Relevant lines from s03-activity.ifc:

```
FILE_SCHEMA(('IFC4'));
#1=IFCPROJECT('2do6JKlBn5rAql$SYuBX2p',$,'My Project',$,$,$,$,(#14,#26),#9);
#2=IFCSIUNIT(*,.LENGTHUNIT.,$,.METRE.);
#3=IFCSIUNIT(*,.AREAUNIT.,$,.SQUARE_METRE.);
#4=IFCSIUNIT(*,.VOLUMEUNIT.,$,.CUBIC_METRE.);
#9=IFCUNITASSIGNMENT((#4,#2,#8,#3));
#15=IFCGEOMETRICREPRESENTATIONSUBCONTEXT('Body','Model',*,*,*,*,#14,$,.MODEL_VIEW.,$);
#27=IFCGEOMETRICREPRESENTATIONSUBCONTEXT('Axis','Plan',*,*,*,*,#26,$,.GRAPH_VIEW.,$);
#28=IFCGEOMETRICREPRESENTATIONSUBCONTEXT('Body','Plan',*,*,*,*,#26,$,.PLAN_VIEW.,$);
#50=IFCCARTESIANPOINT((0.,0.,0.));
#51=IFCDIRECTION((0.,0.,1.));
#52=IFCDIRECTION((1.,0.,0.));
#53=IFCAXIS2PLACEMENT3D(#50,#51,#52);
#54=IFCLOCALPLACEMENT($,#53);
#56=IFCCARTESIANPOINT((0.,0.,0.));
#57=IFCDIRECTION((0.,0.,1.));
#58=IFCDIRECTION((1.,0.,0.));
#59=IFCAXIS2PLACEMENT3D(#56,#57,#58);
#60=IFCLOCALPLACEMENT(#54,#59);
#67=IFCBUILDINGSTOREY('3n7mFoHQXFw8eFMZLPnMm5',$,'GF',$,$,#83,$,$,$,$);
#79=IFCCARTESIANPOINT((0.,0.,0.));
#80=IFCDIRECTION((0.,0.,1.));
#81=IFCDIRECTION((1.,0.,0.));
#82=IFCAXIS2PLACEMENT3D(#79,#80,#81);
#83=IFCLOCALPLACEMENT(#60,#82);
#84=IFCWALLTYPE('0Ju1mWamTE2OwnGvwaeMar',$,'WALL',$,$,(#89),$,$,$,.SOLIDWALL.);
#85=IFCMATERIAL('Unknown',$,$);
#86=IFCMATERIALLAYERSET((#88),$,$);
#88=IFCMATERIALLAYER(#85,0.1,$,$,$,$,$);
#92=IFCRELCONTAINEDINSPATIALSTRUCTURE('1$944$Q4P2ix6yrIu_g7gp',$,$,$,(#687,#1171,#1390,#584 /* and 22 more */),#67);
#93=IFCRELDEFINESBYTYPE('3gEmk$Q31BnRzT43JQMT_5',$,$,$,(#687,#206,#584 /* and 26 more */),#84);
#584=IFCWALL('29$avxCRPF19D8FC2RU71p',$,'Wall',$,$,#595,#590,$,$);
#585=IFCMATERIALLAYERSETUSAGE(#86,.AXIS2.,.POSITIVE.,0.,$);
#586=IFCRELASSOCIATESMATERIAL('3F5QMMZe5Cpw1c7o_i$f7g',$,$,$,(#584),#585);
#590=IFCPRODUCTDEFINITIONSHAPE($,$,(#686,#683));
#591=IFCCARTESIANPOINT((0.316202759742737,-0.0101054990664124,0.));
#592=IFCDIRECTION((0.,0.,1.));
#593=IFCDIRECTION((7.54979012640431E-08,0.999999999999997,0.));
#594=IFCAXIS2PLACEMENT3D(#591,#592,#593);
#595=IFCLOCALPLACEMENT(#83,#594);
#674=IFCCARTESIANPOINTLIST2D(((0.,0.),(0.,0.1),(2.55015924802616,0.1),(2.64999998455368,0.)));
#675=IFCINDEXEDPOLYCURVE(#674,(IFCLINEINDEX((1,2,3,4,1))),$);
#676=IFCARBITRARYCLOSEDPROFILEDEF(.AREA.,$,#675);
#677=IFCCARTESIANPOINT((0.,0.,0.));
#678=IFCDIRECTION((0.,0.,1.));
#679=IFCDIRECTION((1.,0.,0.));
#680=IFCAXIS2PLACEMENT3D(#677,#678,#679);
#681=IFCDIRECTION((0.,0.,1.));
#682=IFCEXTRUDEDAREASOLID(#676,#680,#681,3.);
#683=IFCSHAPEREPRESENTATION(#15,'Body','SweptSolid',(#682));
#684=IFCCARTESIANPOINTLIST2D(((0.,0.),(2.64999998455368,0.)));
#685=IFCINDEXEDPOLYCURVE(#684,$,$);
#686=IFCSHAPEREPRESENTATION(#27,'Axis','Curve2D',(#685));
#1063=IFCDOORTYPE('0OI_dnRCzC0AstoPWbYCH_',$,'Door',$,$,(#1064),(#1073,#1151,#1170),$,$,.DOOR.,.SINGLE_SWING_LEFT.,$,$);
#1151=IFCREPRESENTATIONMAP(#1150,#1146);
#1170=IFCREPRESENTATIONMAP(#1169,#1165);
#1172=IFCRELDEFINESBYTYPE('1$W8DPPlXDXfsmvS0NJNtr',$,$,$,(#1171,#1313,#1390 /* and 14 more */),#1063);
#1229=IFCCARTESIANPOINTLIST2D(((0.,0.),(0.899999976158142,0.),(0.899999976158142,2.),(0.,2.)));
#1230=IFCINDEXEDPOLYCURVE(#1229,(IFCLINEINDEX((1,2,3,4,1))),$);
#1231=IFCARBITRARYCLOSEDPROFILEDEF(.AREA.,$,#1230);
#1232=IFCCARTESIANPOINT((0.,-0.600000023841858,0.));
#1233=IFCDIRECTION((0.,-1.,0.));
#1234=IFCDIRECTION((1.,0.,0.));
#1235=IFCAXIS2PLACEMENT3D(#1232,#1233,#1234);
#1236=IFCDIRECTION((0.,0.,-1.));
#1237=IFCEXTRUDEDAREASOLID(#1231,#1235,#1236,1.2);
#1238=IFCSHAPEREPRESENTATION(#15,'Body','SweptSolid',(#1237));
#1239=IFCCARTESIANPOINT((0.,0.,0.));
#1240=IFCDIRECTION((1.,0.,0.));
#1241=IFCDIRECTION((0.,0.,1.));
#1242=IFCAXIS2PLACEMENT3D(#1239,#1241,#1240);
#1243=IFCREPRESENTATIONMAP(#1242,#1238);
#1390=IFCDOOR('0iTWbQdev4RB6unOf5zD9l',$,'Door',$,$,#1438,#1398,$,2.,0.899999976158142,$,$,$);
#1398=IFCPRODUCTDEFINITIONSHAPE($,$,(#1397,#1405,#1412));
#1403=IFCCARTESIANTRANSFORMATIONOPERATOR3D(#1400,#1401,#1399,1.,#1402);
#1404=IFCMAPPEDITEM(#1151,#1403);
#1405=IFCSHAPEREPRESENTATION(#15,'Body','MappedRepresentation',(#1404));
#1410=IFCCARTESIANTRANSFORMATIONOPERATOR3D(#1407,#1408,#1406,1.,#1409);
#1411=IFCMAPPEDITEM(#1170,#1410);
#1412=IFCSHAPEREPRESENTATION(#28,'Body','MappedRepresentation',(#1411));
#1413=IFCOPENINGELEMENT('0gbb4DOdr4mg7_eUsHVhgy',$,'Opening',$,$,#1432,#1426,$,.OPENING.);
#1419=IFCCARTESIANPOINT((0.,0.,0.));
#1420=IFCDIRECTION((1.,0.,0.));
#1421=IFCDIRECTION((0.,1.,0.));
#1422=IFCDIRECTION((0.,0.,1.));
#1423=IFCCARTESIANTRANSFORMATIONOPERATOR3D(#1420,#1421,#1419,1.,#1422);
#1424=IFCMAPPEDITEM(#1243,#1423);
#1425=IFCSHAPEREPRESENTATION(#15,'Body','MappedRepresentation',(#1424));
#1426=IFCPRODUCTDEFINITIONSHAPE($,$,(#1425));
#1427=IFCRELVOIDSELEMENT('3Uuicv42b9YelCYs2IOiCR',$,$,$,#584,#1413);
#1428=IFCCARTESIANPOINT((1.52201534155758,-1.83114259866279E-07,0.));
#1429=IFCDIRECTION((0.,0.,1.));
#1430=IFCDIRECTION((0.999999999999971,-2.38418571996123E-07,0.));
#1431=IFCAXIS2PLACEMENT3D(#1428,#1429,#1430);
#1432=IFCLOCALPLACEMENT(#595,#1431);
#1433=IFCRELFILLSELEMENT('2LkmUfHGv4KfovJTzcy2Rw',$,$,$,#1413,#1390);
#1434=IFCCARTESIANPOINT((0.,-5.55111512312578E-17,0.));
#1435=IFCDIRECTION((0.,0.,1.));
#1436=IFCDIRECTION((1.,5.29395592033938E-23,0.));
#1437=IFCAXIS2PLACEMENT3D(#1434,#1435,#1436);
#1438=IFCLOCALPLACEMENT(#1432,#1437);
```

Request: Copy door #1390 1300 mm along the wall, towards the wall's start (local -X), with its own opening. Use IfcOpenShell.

```python
import ifcopenshell
import ifcopenshell.api.feature
import ifcopenshell.api.geometry
import ifcopenshell.api.root
import ifcopenshell.geom
import ifcopenshell.util.element
import ifcopenshell.util.placement
import ifcopenshell.util.shape

model = ifcopenshell.open("s03-activity.ifc")
settings = ifcopenshell.geom.settings()


def volume(element):
    """Net volume in cubic metres, openings subtracted."""
    shape = ifcopenshell.geom.create_shape(settings, element)
    return ifcopenshell.util.shape.get_volume(shape.geometry)


door = model.by_id(1390)
opening = door.FillsVoids[0].RelatingOpeningElement
wall = opening.VoidsElements[0].RelatingBuildingElement
before = volume(wall)
shift = ifcopenshell.util.placement.get_local_placement(wall.ObjectPlacement)[:3, 0] * -1.3

# copy_class copies the void relationship, type, container and properties, but no geometry.
new_opening = ifcopenshell.api.root.copy_class(model, product=opening)
new_opening.Representation = ifcopenshell.util.element.copy_deep(
    model, opening.Representation, exclude=["IfcGeometricRepresentationContext", "IfcRepresentationMap"]
)
new_door = ifcopenshell.api.root.copy_class(model, product=door)
new_door.Representation = ifcopenshell.util.element.copy_deep(
    model, door.Representation, exclude=["IfcGeometricRepresentationContext", "IfcRepresentationMap"]
)
ifcopenshell.api.feature.add_filling(model, opening=new_opening, element=new_door)

for old, new in ((opening, new_opening), (door, new_door)):
    matrix = ifcopenshell.util.placement.get_local_placement(old.ObjectPlacement)
    matrix[:3, 3] += shift
    ifcopenshell.api.geometry.edit_object_placement(model, product=new, matrix=matrix, is_si=False)

after = volume(wall)

print(f"wall volume {before:.3f} -> {after:.3f} m3")

model.write("s03-activity_v2.ifc")
```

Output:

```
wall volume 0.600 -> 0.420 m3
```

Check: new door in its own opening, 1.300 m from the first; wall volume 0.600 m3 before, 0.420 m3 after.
